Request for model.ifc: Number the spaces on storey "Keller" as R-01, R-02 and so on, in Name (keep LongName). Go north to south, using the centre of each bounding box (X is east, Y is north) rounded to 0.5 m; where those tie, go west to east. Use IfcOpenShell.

First a look at what the model holds.

```python
import ifcopenshell
import ifcopenshell.util.element
import ifcopenshell.util.placement

model = ifcopenshell.open("model.ifc")
print(model.schema)
storey = next(s for s in model.by_type("IfcBuildingStorey") if s.Name == "Keller")
spaces = [e for e in ifcopenshell.util.element.get_decomposition(storey) if e.is_a("IfcSpace")]
for e in sorted(spaces, key=lambda e: e.id()):
    origin = ifcopenshell.util.placement.get_local_placement(e.ObjectPlacement)[:3, 3]
    print(e.id(), e.Name, e.LongName, origin.round(2) + 0.0, sep=" | ")
```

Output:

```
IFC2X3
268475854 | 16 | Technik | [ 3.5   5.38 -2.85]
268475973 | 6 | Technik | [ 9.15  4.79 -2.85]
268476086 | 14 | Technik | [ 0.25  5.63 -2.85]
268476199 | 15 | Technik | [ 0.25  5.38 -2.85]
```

```python
import ifcopenshell
import ifcopenshell.geom
import ifcopenshell.util.element
import ifcopenshell.util.shape

model = ifcopenshell.open("model.ifc")
settings = ifcopenshell.geom.settings()
settings.set("use-world-coords", True)


def centre(element):
    shape = ifcopenshell.geom.create_shape(settings, element)
    return ifcopenshell.util.shape.get_bbox_centroid(shape.geometry)


storey = next(s for s in model.by_type("IfcBuildingStorey") if s.Name == "Keller")
spaces = [e for e in ifcopenshell.util.element.get_decomposition(storey) if e.is_a("IfcSpace")]

# Insertion points can sit at a corner or the storey origin, so sort by the geometry (in metres).
centres = {e: centre(e) for e in spaces}
spaces.sort(key=lambda e: (-round(centres[e][1] / 0.5), centres[e][0]))

for i, e in enumerate(spaces, start=1):
    number = f"R-{i:02d}"
    e.Name = number
    print(e.id(), number)

model.write("model_edited.ifc")
```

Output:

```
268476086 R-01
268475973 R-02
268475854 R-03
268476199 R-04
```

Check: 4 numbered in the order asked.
